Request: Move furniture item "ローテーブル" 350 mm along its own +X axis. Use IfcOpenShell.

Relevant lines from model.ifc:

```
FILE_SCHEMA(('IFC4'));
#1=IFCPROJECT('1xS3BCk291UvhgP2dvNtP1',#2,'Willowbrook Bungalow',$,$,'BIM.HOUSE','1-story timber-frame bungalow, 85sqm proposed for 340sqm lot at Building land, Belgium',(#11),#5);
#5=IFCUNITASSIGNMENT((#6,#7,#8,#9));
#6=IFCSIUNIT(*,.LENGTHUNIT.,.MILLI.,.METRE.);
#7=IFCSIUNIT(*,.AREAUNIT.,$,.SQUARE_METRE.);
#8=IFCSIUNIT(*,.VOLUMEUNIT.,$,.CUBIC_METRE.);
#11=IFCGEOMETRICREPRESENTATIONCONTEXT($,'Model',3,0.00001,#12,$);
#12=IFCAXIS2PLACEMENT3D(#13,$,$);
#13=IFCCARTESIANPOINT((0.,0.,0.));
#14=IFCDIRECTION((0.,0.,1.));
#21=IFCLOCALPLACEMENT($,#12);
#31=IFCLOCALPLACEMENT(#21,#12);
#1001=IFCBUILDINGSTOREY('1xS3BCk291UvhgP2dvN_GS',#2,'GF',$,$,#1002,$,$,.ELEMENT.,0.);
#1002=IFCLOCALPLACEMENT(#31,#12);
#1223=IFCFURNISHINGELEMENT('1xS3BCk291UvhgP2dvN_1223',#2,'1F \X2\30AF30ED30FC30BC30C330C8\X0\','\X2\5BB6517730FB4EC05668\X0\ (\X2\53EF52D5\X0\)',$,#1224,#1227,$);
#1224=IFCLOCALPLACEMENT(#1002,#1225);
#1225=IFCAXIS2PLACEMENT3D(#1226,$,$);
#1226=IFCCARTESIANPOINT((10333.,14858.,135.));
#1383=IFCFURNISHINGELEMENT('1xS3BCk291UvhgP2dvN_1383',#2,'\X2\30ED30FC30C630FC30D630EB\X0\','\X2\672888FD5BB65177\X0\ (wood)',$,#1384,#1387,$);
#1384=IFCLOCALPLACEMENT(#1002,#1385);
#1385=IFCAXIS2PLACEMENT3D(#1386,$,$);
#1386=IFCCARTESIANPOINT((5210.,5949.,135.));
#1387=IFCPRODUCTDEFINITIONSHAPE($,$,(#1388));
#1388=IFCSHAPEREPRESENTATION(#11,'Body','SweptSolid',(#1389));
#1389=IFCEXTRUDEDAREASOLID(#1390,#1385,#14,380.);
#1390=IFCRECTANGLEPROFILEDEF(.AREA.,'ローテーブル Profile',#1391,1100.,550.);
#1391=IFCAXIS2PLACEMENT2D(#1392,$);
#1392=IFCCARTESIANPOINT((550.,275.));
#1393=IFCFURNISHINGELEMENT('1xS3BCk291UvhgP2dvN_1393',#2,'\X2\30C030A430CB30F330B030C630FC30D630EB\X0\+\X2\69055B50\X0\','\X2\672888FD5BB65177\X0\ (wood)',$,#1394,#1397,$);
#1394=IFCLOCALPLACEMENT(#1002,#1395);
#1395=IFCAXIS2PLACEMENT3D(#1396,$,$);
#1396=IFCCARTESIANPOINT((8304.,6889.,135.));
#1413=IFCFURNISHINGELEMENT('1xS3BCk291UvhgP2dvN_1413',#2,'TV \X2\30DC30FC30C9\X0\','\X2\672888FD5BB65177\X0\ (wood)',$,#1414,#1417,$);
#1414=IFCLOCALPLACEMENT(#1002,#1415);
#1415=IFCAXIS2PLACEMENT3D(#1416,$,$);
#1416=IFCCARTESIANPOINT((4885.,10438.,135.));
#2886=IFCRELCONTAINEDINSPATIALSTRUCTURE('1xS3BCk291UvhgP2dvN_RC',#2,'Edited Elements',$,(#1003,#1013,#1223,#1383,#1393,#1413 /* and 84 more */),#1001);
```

```python
import ifcopenshell
import ifcopenshell.api.geometry
import ifcopenshell.util.placement
import ifcopenshell.util.unit

model = ifcopenshell.open("model.ifc")
unit_scale = ifcopenshell.util.unit.calculate_unit_scale(model)

item = model.by_guid("1xS3BCk291UvhgP2dvN_1383")
matrix = ifcopenshell.util.placement.get_local_placement(item.ObjectPlacement)
matrix[:3, 3] += matrix[:3, 0] * 0.35 / unit_scale
ifcopenshell.api.geometry.edit_object_placement(model, product=item, matrix=matrix, is_si=False)

print(ifcopenshell.util.placement.get_local_placement(item.ObjectPlacement).round(3) + 0.0)

model.write("model_v2.ifc")
```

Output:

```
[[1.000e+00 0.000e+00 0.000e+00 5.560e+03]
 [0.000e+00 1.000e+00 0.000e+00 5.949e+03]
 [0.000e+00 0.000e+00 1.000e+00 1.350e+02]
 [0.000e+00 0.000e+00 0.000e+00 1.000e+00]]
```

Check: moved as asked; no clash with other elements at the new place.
